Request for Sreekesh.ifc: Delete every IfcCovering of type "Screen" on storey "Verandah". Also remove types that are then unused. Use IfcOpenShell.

First a look at what the model holds.

```python
import ifcopenshell
import ifcopenshell.util.element

model = ifcopenshell.open("Sreekesh.ifc")
print(model.schema)
storey = next(s for s in model.by_type("IfcBuildingStorey") if s.Name == "Verandah")
coverings = [e for e in ifcopenshell.util.element.get_decomposition(storey) if e.is_a("IfcCovering")]
seen = {}
for e in coverings:
    element_type = ifcopenshell.util.element.get_type(e)
    name = element_type.Name if element_type not in (None, e) else None
    seen[name] = seen.get(name, 0) + 1
for name, count in sorted(seen.items(), key=str):
    print(count, "x", name)
```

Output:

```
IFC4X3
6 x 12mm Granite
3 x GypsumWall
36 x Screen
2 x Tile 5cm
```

```python
import ifcopenshell
import ifcopenshell.api.root
import ifcopenshell.util.element

model = ifcopenshell.open("Sreekesh.ifc")

storey = next(s for s in model.by_type("IfcBuildingStorey") if s.Name == "Verandah")
coverings = [e for e in ifcopenshell.util.element.get_decomposition(storey) if e.is_a("IfcCovering")]
targets = [e for e in coverings if (t := ifcopenshell.util.element.get_type(e)) not in (None, e) and t.Name == "Screen"]
types = {ifcopenshell.util.element.get_type(e) for e in targets} - {None, *targets}

for e in targets:
    ifcopenshell.api.root.remove_product(model, product=e)
print(len(targets), "removed")

unused = [t for t in types if not ifcopenshell.util.element.get_types(t)]
for t in unused:
    ifcopenshell.api.root.remove_product(model, product=t)
print(len(unused), "unused types removed")

model.write("Sreekesh-out.ifc")
```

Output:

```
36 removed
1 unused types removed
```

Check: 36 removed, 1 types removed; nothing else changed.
